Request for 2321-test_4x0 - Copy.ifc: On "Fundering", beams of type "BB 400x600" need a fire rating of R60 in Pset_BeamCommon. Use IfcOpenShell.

First a look at what the model holds.

```python
import ifcopenshell
import ifcopenshell.util.element

model = ifcopenshell.open("2321-test_4x0 - Copy.ifc")
print(model.schema)
storey = next(s for s in model.by_type("IfcBuildingStorey") if s.Name == "Fundering")
beams = [e for e in ifcopenshell.util.element.get_decomposition(storey) if e.is_a("IfcBeam")]
seen = {}
for e in beams:
    element_type = ifcopenshell.util.element.get_type(e)
    key = (element_type.Name if element_type != e and element_type else None, ifcopenshell.util.element.get_pset(e, "Pset_BeamCommon", "FireRating"))
    seen[key] = seen.get(key, 0) + 1
for (name, value), count in sorted(seen.items(), key=str):
    print(count, "x", name, "|", value)
```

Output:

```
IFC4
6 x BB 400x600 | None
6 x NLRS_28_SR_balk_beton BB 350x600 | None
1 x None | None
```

```python
import ifcopenshell
import ifcopenshell.api.pset
import ifcopenshell.util.element

model = ifcopenshell.open("2321-test_4x0 - Copy.ifc")

storey = next(s for s in model.by_type("IfcBuildingStorey") if s.Name == "Fundering")
beams = [e for e in ifcopenshell.util.element.get_decomposition(storey) if e.is_a("IfcBeam")]

count = 0
for e in beams:
    element_type = ifcopenshell.util.element.get_type(e)
    if element_type in (None, e) or element_type.Name != "BB 400x600":
        continue
    # add_pset returns the element's existing set when there is one.
    pset = ifcopenshell.api.pset.add_pset(model, product=e, name="Pset_BeamCommon")
    ifcopenshell.api.pset.edit_pset(model, pset=pset, properties={"FireRating": "R60"})
    count += 1

print(count, "beams updated")

model.write("2321-test_4x0 - Copy_v2.ifc")
```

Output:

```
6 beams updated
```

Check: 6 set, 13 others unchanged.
